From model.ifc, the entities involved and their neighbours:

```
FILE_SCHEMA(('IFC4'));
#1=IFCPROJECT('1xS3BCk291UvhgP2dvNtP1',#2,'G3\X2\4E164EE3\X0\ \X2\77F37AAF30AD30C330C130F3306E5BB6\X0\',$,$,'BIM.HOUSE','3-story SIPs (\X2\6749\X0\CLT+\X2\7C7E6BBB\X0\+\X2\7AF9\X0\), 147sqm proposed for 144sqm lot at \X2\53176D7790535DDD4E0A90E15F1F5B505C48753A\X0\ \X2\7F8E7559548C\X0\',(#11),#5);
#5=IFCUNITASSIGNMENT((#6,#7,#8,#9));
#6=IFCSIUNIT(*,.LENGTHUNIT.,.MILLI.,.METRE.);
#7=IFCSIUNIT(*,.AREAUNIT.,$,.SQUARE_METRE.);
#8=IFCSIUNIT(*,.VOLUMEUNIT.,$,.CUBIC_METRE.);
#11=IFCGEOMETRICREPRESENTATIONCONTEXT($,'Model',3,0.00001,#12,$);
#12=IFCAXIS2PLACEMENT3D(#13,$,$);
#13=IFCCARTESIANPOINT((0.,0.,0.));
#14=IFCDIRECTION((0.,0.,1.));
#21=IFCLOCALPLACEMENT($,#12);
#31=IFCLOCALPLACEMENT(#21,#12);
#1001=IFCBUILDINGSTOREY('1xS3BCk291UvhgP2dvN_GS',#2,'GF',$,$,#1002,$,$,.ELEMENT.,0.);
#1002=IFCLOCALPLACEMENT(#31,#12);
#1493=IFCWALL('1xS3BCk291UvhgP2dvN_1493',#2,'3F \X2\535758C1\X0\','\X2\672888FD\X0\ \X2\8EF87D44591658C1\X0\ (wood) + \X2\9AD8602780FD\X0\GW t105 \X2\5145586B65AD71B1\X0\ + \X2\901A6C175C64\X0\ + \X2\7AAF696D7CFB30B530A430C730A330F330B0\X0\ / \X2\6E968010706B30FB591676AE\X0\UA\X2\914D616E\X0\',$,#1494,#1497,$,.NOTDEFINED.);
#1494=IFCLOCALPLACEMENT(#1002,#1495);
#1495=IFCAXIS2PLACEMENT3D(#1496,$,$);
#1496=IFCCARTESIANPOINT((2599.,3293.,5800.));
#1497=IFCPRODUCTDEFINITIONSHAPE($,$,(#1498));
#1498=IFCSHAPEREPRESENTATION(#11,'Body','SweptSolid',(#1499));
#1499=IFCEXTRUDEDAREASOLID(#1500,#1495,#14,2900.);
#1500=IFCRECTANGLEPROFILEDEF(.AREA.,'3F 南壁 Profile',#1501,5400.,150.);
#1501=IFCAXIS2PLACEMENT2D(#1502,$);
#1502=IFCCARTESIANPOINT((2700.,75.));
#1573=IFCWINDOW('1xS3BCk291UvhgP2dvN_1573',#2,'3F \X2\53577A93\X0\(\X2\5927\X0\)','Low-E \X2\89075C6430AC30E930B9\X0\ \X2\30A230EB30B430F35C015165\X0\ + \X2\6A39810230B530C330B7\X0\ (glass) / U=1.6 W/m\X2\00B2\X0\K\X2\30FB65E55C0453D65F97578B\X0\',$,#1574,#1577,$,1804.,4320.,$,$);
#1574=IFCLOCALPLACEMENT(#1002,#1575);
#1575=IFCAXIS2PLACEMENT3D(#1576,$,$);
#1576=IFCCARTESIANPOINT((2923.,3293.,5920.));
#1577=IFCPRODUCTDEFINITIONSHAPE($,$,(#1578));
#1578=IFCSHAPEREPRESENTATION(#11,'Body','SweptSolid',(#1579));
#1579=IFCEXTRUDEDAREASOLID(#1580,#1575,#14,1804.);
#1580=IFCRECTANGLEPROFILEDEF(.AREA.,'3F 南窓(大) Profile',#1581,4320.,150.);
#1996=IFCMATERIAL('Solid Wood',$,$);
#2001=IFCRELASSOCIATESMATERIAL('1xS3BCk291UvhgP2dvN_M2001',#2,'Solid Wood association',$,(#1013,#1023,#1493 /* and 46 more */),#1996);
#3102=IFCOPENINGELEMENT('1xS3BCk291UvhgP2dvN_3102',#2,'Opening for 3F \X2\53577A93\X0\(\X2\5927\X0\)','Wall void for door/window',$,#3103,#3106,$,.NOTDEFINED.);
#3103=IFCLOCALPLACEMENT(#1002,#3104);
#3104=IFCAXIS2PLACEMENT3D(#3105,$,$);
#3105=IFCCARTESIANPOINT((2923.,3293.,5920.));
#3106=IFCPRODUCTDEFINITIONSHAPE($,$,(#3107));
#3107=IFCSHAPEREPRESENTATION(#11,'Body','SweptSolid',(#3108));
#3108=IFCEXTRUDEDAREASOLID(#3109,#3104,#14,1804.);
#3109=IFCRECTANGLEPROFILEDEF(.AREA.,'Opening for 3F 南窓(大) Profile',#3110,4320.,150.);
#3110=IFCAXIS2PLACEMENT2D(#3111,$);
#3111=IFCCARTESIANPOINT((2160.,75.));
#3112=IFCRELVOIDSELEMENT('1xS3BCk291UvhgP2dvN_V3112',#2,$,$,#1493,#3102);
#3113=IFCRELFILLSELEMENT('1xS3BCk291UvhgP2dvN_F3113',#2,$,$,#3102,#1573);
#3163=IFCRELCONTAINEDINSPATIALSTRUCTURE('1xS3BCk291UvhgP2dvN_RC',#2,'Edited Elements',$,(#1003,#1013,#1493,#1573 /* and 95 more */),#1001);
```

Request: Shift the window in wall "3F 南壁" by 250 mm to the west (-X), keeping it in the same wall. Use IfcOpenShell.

```python
import ifcopenshell
import ifcopenshell.api.geometry
import ifcopenshell.util.placement
import ifcopenshell.util.unit

model = ifcopenshell.open("model.ifc")
unit_scale = ifcopenshell.util.unit.calculate_unit_scale(model)

window = model.by_guid("1xS3BCk291UvhgP2dvN_1573")
opening = window.FillsVoids[0].RelatingOpeningElement
wall = opening.VoidsElements[0].RelatingBuildingElement

wall_matrix = ifcopenshell.util.placement.get_local_placement(wall.ObjectPlacement)
shift = wall_matrix[:3, 0] * -0.25 / unit_scale
before = ifcopenshell.util.placement.get_local_placement(window.ObjectPlacement)[:3, 3].copy()

# The window is not placed relative to its opening, so move both.
for product in (opening, window):
    matrix = ifcopenshell.util.placement.get_local_placement(product.ObjectPlacement)
    matrix[:3, 3] += shift
    ifcopenshell.api.geometry.edit_object_placement(model, product=product, matrix=matrix, is_si=False)

after = ifcopenshell.util.placement.get_local_placement(window.ObjectPlacement)[:3, 3]
print("window moved by", (after - before).round(3) + 0.0)

model.write("model-out.ifc")
```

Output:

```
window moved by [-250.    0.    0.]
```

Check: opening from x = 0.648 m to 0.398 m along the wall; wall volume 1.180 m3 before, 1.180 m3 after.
